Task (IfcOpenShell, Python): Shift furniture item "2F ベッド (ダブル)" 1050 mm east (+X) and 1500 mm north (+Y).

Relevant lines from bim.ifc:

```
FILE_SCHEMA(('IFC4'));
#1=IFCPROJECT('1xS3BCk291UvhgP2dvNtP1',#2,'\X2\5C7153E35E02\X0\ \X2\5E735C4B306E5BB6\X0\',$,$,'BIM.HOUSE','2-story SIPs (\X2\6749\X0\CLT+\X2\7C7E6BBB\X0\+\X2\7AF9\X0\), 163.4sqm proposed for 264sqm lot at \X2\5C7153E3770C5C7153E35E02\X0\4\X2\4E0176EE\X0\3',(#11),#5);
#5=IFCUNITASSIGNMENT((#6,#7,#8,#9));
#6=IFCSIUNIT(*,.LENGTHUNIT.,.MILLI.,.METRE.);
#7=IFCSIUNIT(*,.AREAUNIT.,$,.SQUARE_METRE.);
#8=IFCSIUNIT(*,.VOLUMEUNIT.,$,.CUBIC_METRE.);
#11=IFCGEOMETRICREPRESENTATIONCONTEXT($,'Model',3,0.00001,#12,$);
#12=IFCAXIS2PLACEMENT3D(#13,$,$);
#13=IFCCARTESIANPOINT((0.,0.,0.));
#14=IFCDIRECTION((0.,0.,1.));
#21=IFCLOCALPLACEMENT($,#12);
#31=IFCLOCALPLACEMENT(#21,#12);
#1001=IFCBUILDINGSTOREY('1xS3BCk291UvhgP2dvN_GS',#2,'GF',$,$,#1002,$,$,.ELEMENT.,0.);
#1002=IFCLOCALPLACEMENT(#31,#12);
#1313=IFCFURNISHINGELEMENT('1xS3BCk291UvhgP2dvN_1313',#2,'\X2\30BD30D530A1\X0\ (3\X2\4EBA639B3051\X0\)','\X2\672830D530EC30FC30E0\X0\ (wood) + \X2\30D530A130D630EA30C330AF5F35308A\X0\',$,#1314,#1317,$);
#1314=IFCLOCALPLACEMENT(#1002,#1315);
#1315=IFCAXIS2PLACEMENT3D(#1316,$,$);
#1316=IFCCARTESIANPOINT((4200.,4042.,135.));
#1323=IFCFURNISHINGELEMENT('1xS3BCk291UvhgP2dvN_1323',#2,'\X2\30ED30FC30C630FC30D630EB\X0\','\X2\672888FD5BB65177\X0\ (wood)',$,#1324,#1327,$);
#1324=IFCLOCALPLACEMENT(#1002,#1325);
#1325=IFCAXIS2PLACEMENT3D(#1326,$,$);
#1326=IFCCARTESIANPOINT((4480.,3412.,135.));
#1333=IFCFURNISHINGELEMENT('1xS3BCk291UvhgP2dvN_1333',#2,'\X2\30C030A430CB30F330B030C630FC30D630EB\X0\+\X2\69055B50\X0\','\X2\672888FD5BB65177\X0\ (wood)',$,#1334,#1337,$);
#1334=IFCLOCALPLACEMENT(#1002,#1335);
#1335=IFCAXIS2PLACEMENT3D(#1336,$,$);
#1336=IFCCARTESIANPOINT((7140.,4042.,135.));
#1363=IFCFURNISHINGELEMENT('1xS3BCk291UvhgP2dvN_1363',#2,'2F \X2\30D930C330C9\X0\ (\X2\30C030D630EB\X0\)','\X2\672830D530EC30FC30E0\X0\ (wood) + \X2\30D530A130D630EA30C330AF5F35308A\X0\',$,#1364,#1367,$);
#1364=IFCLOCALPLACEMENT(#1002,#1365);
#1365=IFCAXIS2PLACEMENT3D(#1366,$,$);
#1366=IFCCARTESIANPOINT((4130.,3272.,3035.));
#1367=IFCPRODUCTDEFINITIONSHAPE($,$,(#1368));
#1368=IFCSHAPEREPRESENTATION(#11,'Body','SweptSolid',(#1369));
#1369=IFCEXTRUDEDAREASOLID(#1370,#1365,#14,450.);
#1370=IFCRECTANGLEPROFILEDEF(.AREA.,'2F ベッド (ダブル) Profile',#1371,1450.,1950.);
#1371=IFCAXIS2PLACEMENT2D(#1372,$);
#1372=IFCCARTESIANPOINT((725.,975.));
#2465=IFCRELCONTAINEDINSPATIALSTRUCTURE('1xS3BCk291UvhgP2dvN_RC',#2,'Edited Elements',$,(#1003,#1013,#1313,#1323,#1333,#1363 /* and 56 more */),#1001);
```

```python
import ifcopenshell
import ifcopenshell.api.geometry
import ifcopenshell.util.placement

model = ifcopenshell.open("bim.ifc")

item = model.by_id(1363)
matrix = ifcopenshell.util.placement.get_local_placement(item.ObjectPlacement)
matrix[0, 3] += 1050.0
matrix[1, 3] += 1500.0
ifcopenshell.api.geometry.edit_object_placement(model, product=item, matrix=matrix, is_si=False)

print(ifcopenshell.util.placement.get_local_placement(item.ObjectPlacement).round(3) + 0.0)

model.write("bim_rev.ifc")
```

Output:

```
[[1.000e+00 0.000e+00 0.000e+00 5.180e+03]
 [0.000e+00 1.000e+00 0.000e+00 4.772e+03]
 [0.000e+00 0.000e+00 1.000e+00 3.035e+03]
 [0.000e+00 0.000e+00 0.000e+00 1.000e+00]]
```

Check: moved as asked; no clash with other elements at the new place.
